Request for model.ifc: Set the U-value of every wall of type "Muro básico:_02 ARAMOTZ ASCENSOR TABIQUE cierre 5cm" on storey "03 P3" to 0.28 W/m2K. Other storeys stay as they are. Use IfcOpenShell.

First a look at what the model holds.

```python
import ifcopenshell
import ifcopenshell.util.element

model = ifcopenshell.open("model.ifc")
print(model.schema)
storey = next(s for s in model.by_type("IfcBuildingStorey") if s.Name == "03 P3")
walls = [e for e in ifcopenshell.util.element.get_decomposition(storey) if e.is_a("IfcWall")]
seen = {}
for e in walls:
    element_type = ifcopenshell.util.element.get_type(e)
    key = (element_type.Name if element_type != e and element_type else None, ifcopenshell.util.element.get_pset(e, "Pset_WallCommon", "ThermalTransmittance"))
    seen[key] = seen.get(key, 0) + 1
for (name, value), count in sorted(seen.items(), key=str):
    print(count, "x", name, "|", value)
```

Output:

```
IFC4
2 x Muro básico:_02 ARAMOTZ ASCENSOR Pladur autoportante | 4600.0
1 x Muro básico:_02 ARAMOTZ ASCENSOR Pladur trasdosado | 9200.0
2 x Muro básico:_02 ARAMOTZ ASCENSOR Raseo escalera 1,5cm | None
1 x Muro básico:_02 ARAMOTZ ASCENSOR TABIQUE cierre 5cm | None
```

```python
import ifcopenshell
import ifcopenshell.api.pset
import ifcopenshell.util.element

model = ifcopenshell.open("model.ifc")

storey = next(s for s in model.by_type("IfcBuildingStorey") if s.Name == "03 P3")
walls = [e for e in ifcopenshell.util.element.get_decomposition(storey) if e.is_a("IfcWall")]

count = 0
for e in walls:
    element_type = ifcopenshell.util.element.get_type(e)
    if element_type in (None, e) or element_type.Name != "Muro básico:_02 ARAMOTZ ASCENSOR TABIQUE cierre 5cm":
        continue
    # add_pset returns the element's existing set when there is one.
    pset = ifcopenshell.api.pset.add_pset(model, product=e, name="Pset_WallCommon")
    ifcopenshell.api.pset.edit_pset(model, pset=pset, properties={"ThermalTransmittance": 0.28})
    count += 1

print(count, "walls updated")

model.write("model_updated.ifc")
```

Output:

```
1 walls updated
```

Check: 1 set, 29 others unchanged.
